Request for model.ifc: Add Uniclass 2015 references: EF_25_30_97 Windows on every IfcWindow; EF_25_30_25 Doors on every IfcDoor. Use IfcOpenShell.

First a look at what the model holds.

```python
import ifcopenshell

model = ifcopenshell.open("model.ifc")
print(model.schema)
print("classifications:", [c.Name for c in model.by_type("IfcClassification")])
for ifc_class in ("IfcDoor", "IfcRoof", "IfcStair", "IfcWall", "IfcWindow"):
    print(ifc_class, len(model.by_type(ifc_class)))
```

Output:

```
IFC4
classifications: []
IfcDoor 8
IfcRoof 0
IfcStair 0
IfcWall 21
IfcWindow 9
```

```python
import ifcopenshell
import ifcopenshell.api.classification

model = ifcopenshell.open("model.ifc")

system = ifcopenshell.api.classification.add_classification(model, classification="Uniclass 2015")

codes = {
    "IfcWindow": ("EF_25_30_97", "Windows"),
    "IfcDoor": ("EF_25_30_25", "Doors"),
}
for ifc_class, (code, name) in codes.items():
    products = model.by_type(ifc_class)
    ifcopenshell.api.classification.add_reference(
        model, products=products, classification=system, identification=code, name=name
    )
    print(code, len(products))

model.write("model_edited.ifc")
```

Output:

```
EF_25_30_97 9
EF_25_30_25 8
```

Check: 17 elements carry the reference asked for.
